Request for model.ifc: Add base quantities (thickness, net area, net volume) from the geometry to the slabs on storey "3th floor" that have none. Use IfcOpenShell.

First a look at what the model holds.

```python
import ifcopenshell
import ifcopenshell.util.element
import ifcopenshell.util.unit

model = ifcopenshell.open("model.ifc")
print(model.schema)
for unit_type in ("LENGTHUNIT", "AREAUNIT", "VOLUMEUNIT"):
    print(unit_type, ifcopenshell.util.unit.calculate_unit_scale(model, unit_type))
storey = next(s for s in model.by_type("IfcBuildingStorey") if s.Name == "3th floor")
slabs = [e for e in ifcopenshell.util.element.get_decomposition(storey) if e.is_a("IfcSlab")]
for e in sorted(slabs, key=lambda e: e.id()):
    print(e.id(), e.is_a(), e.Name, list(ifcopenshell.util.element.get_psets(e, qtos_only=True)), sep=" | ")
```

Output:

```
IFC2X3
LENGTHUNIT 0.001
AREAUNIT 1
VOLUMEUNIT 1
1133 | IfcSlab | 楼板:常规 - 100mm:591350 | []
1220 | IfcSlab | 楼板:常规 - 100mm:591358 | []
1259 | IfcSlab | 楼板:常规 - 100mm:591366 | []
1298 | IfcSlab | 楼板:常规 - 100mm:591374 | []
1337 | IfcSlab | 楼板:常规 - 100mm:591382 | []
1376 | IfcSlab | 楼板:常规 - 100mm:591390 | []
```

```python
import ifcopenshell
import ifcopenshell.api.pset
import ifcopenshell.geom
import ifcopenshell.util.element
import ifcopenshell.util.shape
import ifcopenshell.util.unit

model = ifcopenshell.open("model.ifc")
unit_scale = ifcopenshell.util.unit.calculate_unit_scale(model)
area_scale = ifcopenshell.util.unit.calculate_unit_scale(model, "AREAUNIT")
volume_scale = ifcopenshell.util.unit.calculate_unit_scale(model, "VOLUMEUNIT")
settings = ifcopenshell.geom.settings()

storey = next(s for s in model.by_type("IfcBuildingStorey") if s.Name == "3th floor")
slabs = [e for e in ifcopenshell.util.element.get_decomposition(storey) if e.is_a("IfcSlab")]

for e in sorted(slabs, key=lambda e: e.id()):
    if ifcopenshell.util.element.get_psets(e, qtos_only=True, should_inherit=False):
        continue
    # Geometry comes back in metres, in the element's own axes.
    shape = ifcopenshell.geom.create_shape(settings, e)
    values = {
        "Width": ifcopenshell.util.shape.get_z(shape.geometry) / unit_scale,
        "NetArea": ifcopenshell.util.shape.get_footprint_area(shape.geometry) / area_scale,
        "NetVolume": ifcopenshell.util.shape.get_volume(shape.geometry) / volume_scale,
    }
    qto = ifcopenshell.api.pset.add_qto(model, product=e, name="BaseQuantities")
    ifcopenshell.api.pset.edit_qto(model, qto=qto, properties=values)
    print(e.id(), {k: round(v, 3) for k, v in values.items()})

model.write("model_rev.ifc")
```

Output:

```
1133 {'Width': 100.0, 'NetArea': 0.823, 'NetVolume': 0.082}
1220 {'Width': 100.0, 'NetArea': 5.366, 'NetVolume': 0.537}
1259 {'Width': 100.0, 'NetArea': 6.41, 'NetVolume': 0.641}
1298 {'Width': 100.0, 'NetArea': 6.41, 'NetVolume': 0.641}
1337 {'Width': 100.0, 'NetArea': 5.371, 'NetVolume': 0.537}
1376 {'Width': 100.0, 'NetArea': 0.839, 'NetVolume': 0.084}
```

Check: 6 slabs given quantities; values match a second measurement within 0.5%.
